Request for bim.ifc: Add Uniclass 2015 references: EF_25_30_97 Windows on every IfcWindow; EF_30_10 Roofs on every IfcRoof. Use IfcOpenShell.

First a look at what the model holds.

```python
import ifcopenshell

model = ifcopenshell.open("bim.ifc")
print(model.schema)
print("classifications:", [c.Name for c in model.by_type("IfcClassification")])
for ifc_class in ("IfcDoor", "IfcRoof", "IfcStair", "IfcWall", "IfcWindow"):
    print(ifc_class, len(model.by_type(ifc_class)))
```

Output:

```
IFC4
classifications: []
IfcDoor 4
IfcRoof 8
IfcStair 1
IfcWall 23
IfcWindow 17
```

```python
import ifcopenshell
import ifcopenshell.api.classification

model = ifcopenshell.open("bim.ifc")

system = ifcopenshell.api.classification.add_classification(model, classification="Uniclass 2015")

codes = {
    "IfcWindow": ("EF_25_30_97", "Windows"),
    "IfcRoof": ("EF_30_10", "Roofs"),
}
for ifc_class, (code, name) in codes.items():
    products = model.by_type(ifc_class)
    ifcopenshell.api.classification.add_reference(
        model, products=products, classification=system, identification=code, name=name
    )
    print(code, len(products))

model.write("bim_rev.ifc")
```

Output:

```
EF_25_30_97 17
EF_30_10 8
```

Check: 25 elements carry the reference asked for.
